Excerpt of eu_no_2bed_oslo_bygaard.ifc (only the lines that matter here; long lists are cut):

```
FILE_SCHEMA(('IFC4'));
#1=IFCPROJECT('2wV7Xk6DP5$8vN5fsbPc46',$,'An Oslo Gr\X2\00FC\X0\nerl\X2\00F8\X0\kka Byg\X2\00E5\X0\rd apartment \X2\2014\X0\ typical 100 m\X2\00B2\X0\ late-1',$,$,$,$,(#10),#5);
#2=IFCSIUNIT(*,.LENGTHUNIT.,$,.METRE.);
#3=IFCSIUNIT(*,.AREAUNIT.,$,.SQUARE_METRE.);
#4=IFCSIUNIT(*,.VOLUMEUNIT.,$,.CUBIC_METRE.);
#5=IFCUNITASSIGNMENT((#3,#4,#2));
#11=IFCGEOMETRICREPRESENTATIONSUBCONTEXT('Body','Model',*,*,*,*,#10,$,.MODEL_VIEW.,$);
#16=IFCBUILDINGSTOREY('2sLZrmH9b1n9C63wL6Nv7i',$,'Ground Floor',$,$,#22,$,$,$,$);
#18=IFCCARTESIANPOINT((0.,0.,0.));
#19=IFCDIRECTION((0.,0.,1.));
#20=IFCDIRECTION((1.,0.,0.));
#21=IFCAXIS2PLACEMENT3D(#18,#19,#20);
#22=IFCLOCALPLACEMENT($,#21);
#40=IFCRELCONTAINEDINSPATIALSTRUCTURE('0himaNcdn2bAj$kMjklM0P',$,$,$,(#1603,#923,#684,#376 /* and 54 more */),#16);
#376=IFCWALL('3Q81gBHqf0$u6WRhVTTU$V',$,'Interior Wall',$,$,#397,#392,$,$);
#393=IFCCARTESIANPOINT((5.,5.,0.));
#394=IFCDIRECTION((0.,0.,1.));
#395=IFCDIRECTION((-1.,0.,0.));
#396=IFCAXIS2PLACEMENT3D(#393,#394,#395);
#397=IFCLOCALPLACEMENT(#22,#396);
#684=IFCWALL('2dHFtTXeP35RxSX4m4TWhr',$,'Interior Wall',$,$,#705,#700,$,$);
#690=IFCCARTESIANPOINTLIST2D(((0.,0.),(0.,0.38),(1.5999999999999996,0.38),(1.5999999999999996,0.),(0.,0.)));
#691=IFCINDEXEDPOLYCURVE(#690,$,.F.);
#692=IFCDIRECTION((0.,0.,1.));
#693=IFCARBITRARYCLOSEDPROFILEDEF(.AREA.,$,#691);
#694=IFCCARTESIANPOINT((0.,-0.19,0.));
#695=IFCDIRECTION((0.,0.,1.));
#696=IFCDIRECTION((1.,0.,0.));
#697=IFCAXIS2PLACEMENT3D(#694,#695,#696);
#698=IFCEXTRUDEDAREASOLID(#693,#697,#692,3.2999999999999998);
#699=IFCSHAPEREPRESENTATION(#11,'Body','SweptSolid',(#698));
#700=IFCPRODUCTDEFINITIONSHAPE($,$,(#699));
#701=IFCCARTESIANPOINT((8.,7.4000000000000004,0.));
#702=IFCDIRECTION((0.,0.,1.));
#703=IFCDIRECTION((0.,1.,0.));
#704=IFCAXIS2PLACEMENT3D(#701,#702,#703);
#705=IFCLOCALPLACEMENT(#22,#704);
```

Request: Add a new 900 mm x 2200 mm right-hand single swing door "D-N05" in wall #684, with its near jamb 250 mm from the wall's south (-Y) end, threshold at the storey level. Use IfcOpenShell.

```python
import numpy as np
import ifcopenshell
import ifcopenshell.api.feature
import ifcopenshell.api.geometry
import ifcopenshell.api.root
import ifcopenshell.api.spatial
import ifcopenshell.geom
import ifcopenshell.util.element
import ifcopenshell.util.placement
import ifcopenshell.util.representation
import ifcopenshell.util.shape
import ifcopenshell.util.unit

model = ifcopenshell.open("eu_no_2bed_oslo_bygaard.ifc")
unit_scale = ifcopenshell.util.unit.calculate_unit_scale(model)
settings = ifcopenshell.geom.settings()


def volume(element):
    """Net volume in cubic metres, openings subtracted."""
    shape = ifcopenshell.geom.create_shape(settings, element)
    return ifcopenshell.util.shape.get_volume(shape.geometry)


wall = model.by_guid("2dHFtTXeP35RxSX4m4TWhr")
storey = ifcopenshell.util.element.get_container(wall, ifc_class="IfcBuildingStorey")
context = ifcopenshell.util.representation.get_context(model, "Model", "Body", "MODEL_VIEW")
before = volume(wall)

width, height, from_end, sill = 0.9, 2.2, 0.25, 0.0  # metres

# The wall runs along its own X axis, and the end named is its -X end.
wall_shape = ifcopenshell.geom.create_shape(settings, wall)
x, y, z = ifcopenshell.util.shape.get_vertices(wall_shape.geometry).T
start = x.min() + from_end
face, thickness = float(y.min()), float(y.max() - y.min())
wall_matrix = ifcopenshell.util.placement.get_local_placement(wall.ObjectPlacement)
level = ifcopenshell.util.placement.get_local_placement(storey.ObjectPlacement)[2, 3]


def in_wall(x, y):
    """Placement at x, y metres in the wall's axes, at sill height."""
    matrix = wall_matrix.copy()
    matrix[:, 3] = wall_matrix @ np.array([x / unit_scale, y / unit_scale, 0.0, 1.0])
    matrix[2, 3] = level + sill / unit_scale
    return matrix


# Opening: a box that overshoots both wall faces by 50 mm.
opening = ifcopenshell.api.root.create_entity(model, ifc_class="IfcOpeningElement", predefined_type="OPENING")
box = ifcopenshell.api.geometry.add_wall_representation(
    model, context=context, length=width, height=height, thickness=thickness + 0.1
)
ifcopenshell.api.geometry.assign_representation(model, product=opening, representation=box)
ifcopenshell.api.geometry.edit_object_placement(model, product=opening, matrix=in_wall(start, face - 0.05), is_si=False)
ifcopenshell.api.feature.add_feature(model, feature=opening, element=wall)

door = ifcopenshell.api.root.create_entity(model, ifc_class="IfcDoor", name="D-N05", predefined_type="DOOR")
door.OverallWidth, door.OverallHeight = width / unit_scale, height / unit_scale
door.OperationType = "SINGLE_SWING_RIGHT"
body = ifcopenshell.api.geometry.add_door_representation(
    model,
    context=context,
    overall_width=door.OverallWidth,
    overall_height=door.OverallHeight,
    operation_type="SINGLE_SWING_RIGHT",
    lining_properties={"LiningDepth": thickness / unit_scale, "ThresholdDepth": thickness / unit_scale},
)
ifcopenshell.api.geometry.assign_representation(model, product=door, representation=body)
ifcopenshell.api.spatial.assign_container(model, products=[door], relating_structure=storey)
ifcopenshell.api.feature.add_filling(model, opening=opening, element=door)

# The lining spans the wall, so the door starts at the wall face.
ifcopenshell.api.geometry.edit_object_placement(model, product=door, matrix=in_wall(start, face), is_si=False)

after = volume(wall)

print(f"wall volume {before:.3f} -> {after:.3f} m3")

model.write("eu_no_2bed_oslo_bygaard_updated.ifc")
```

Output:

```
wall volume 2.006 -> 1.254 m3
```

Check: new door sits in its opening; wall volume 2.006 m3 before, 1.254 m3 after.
